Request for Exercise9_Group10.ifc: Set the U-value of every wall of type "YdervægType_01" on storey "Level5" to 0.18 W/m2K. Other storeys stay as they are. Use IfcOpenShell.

First a look at what the model holds.

```python
import ifcopenshell
import ifcopenshell.util.element

model = ifcopenshell.open("Exercise9_Group10.ifc")
print(model.schema)
storey = next(s for s in model.by_type("IfcBuildingStorey") if s.Name == "Level5")
walls = [e for e in ifcopenshell.util.element.get_decomposition(storey) if e.is_a("IfcWall")]
seen = {}
for e in walls:
    element_type = ifcopenshell.util.element.get_type(e)
    key = (element_type.Name if element_type != e and element_type else None, ifcopenshell.util.element.get_pset(e, "Pset_WallCommon", "ThermalTransmittance"))
    seen[key] = seen.get(key, 0) + 1
for (name, value), count in sorted(seen.items(), key=str):
    print(count, "x", name, "|", value)
```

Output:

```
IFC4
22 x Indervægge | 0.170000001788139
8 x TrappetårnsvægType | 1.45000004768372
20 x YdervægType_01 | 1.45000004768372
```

```python
import ifcopenshell
import ifcopenshell.api.pset
import ifcopenshell.util.element

model = ifcopenshell.open("Exercise9_Group10.ifc")

storey = next(s for s in model.by_type("IfcBuildingStorey") if s.Name == "Level5")
walls = [e for e in ifcopenshell.util.element.get_decomposition(storey) if e.is_a("IfcWall")]

count = 0
for e in walls:
    element_type = ifcopenshell.util.element.get_type(e)
    if element_type in (None, e) or element_type.Name != "YdervægType_01":
        continue
    # add_pset returns the element's existing set when there is one.
    pset = ifcopenshell.api.pset.add_pset(model, product=e, name="Pset_WallCommon")
    ifcopenshell.api.pset.edit_pset(model, pset=pset, properties={"ThermalTransmittance": 0.18})
    count += 1

print(count, "walls updated")

model.write("Exercise9_Group10_v2.ifc")
```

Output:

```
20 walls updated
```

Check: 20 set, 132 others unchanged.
